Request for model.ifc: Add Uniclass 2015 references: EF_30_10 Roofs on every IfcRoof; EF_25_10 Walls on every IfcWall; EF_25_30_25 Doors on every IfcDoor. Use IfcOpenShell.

First a look at what the model holds.

```python
import ifcopenshell

model = ifcopenshell.open("model.ifc")
print(model.schema)
print("classifications:", [c.Name for c in model.by_type("IfcClassification")])
for ifc_class in ("IfcDoor", "IfcRoof", "IfcStair", "IfcWall", "IfcWindow"):
    print(ifc_class, len(model.by_type(ifc_class)))
```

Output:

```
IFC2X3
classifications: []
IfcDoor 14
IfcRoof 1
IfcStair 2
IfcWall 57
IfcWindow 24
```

```python
import ifcopenshell
import ifcopenshell.api.classification

model = ifcopenshell.open("model.ifc")

# IFC2X3 requires Source and Edition and has no link from the project to the system.
system = model.create_entity("IfcClassification", Source="NBS", Edition="2015", Name="Uniclass 2015")

codes = {
    "IfcRoof": ("EF_30_10", "Roofs"),
    "IfcWall": ("EF_25_10", "Walls"),
    "IfcDoor": ("EF_25_30_25", "Doors"),
}
for ifc_class, (code, name) in codes.items():
    products = model.by_type(ifc_class)
    ifcopenshell.api.classification.add_reference(
        model, products=products, classification=system, identification=code, name=name
    )
    print(code, len(products))

model.write("model_updated.ifc")
```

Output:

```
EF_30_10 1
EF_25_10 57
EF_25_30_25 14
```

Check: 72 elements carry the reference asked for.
